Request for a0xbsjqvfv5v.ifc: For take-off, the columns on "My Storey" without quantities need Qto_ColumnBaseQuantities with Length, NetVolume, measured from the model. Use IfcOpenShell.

First a look at what the model holds.

```python
import ifcopenshell
import ifcopenshell.util.element
import ifcopenshell.util.unit

model = ifcopenshell.open("a0xbsjqvfv5v.ifc")
print(model.schema)
for unit_type in ("LENGTHUNIT", "AREAUNIT", "VOLUMEUNIT"):
    print(unit_type, ifcopenshell.util.unit.calculate_unit_scale(model, unit_type))
storey = next(s for s in model.by_type("IfcBuildingStorey") if s.Name == "My Storey")
columns = [e for e in ifcopenshell.util.element.get_decomposition(storey) if e.is_a("IfcColumn")]
for e in sorted(columns, key=lambda e: e.id()):
    print(e.id(), e.is_a(), e.Name, list(ifcopenshell.util.element.get_psets(e, qtos_only=True)), sep=" | ")
```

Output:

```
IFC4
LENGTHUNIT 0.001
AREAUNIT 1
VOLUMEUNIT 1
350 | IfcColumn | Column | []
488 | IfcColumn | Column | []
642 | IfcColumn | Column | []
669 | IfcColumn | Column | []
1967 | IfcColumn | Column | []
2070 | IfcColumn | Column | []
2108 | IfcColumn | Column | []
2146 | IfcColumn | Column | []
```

```python
import ifcopenshell
import ifcopenshell.api.pset
import ifcopenshell.geom
import ifcopenshell.util.element
import ifcopenshell.util.shape
import ifcopenshell.util.unit

model = ifcopenshell.open("a0xbsjqvfv5v.ifc")
unit_scale = ifcopenshell.util.unit.calculate_unit_scale(model)
volume_scale = ifcopenshell.util.unit.calculate_unit_scale(model, "VOLUMEUNIT")
settings = ifcopenshell.geom.settings()

storey = next(s for s in model.by_type("IfcBuildingStorey") if s.Name == "My Storey")
columns = [e for e in ifcopenshell.util.element.get_decomposition(storey) if e.is_a("IfcColumn")]

for e in sorted(columns, key=lambda e: e.id()):
    if ifcopenshell.util.element.get_psets(e, qtos_only=True, should_inherit=False):
        continue
    # Geometry comes back in metres, in the element's own axes.
    shape = ifcopenshell.geom.create_shape(settings, e)
    values = {
        "Length": ifcopenshell.util.shape.get_z(shape.geometry) / unit_scale,
        "NetVolume": ifcopenshell.util.shape.get_volume(shape.geometry) / volume_scale,
    }
    qto = ifcopenshell.api.pset.add_qto(model, product=e, name="Qto_ColumnBaseQuantities")
    ifcopenshell.api.pset.edit_qto(model, qto=qto, properties=values)
    print(e.id(), {k: round(v, 3) for k, v in values.items()})

model.write("a0xbsjqvfv5v-out.ifc")
```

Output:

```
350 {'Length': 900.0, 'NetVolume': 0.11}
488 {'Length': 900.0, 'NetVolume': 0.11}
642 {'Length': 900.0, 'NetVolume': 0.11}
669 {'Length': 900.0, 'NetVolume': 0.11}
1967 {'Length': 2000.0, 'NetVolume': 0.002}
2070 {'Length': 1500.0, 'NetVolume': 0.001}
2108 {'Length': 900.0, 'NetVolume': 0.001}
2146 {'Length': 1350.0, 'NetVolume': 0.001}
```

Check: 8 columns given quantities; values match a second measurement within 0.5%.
